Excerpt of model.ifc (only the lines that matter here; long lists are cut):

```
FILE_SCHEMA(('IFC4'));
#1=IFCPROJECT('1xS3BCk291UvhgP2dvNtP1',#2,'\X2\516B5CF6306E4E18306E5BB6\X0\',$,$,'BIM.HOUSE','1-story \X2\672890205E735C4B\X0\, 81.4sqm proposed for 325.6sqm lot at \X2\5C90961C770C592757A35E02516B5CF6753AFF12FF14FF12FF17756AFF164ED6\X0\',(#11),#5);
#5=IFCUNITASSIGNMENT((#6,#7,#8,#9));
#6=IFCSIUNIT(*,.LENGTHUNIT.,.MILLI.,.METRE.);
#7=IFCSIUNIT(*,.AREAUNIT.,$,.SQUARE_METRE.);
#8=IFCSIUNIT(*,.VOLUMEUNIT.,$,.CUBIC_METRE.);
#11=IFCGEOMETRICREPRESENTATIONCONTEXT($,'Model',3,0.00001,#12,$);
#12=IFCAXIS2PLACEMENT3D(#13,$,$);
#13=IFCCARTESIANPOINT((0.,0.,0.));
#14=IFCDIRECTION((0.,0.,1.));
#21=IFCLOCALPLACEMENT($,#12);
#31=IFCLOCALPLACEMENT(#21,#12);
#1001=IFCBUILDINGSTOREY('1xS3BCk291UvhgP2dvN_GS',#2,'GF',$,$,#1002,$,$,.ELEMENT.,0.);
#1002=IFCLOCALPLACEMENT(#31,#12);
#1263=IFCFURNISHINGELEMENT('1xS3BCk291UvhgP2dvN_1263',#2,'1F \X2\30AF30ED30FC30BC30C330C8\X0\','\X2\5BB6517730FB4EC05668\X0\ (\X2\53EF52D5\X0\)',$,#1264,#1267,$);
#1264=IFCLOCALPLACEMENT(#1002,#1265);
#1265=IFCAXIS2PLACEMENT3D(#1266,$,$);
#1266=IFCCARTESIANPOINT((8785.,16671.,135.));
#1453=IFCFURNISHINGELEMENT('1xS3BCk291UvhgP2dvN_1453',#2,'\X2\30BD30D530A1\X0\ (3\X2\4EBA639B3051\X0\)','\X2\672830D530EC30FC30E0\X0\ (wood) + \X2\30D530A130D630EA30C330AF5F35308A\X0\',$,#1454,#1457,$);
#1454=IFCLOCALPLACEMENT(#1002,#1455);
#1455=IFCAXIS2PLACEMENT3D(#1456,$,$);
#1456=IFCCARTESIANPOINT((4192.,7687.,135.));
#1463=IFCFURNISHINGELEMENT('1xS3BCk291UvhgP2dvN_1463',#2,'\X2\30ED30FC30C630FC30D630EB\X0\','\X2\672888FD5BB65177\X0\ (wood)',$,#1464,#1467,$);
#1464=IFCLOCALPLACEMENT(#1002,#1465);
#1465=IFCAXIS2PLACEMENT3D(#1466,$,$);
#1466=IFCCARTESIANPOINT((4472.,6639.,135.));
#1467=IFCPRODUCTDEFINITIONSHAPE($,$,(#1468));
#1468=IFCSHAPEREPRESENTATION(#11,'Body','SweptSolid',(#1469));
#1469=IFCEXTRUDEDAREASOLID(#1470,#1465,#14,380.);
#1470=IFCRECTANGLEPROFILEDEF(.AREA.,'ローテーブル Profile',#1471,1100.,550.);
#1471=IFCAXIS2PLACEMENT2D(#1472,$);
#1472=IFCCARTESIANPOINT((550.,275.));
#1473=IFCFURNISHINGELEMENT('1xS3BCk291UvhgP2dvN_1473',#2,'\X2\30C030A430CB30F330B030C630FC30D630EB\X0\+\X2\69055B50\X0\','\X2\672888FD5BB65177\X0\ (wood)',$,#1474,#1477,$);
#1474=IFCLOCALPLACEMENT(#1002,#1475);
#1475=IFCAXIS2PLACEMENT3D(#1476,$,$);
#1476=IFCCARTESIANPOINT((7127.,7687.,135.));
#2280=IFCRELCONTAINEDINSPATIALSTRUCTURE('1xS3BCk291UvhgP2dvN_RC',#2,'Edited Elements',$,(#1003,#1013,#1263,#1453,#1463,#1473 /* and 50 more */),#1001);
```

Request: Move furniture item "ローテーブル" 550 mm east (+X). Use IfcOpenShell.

```python
import ifcopenshell
import ifcopenshell.api.geometry
import ifcopenshell.util.placement

model = ifcopenshell.open("model.ifc")

item = model.by_id(1463)
matrix = ifcopenshell.util.placement.get_local_placement(item.ObjectPlacement)
matrix[0, 3] += 550.0
ifcopenshell.api.geometry.edit_object_placement(model, product=item, matrix=matrix, is_si=False)

print(ifcopenshell.util.placement.get_local_placement(item.ObjectPlacement).round(3) + 0.0)

model.write("model_updated.ifc")
```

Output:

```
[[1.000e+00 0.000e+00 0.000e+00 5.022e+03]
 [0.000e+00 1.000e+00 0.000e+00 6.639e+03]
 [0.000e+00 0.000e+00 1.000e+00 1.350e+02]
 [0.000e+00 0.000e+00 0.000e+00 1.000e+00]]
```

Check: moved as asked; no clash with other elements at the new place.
